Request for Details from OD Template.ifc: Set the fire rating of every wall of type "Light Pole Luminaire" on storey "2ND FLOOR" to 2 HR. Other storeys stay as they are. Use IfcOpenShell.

First a look at what the model holds.

```python
import ifcopenshell
import ifcopenshell.util.element

model = ifcopenshell.open("Details from OD Template.ifc")
print(model.schema)
storey = next(s for s in model.by_type("IfcBuildingStorey") if s.Name == "2ND FLOOR")
walls = [e for e in ifcopenshell.util.element.get_decomposition(storey) if e.is_a("IfcWall")]
seen = {}
for e in walls:
    element_type = ifcopenshell.util.element.get_type(e)
    key = (element_type.Name if element_type != e and element_type else None, ifcopenshell.util.element.get_pset(e, "Pset_WallCommon", "FireRating"))
    seen[key] = seen.get(key, 0) + 1
for (name, value), count in sorted(seen.items(), key=str):
    print(count, "x", name, "|", value)
```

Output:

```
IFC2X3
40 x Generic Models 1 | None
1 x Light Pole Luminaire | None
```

```python
import ifcopenshell
import ifcopenshell.api.pset
import ifcopenshell.util.element

model = ifcopenshell.open("Details from OD Template.ifc")

storey = next(s for s in model.by_type("IfcBuildingStorey") if s.Name == "2ND FLOOR")
walls = [e for e in ifcopenshell.util.element.get_decomposition(storey) if e.is_a("IfcWall")]

count = 0
for e in walls:
    element_type = ifcopenshell.util.element.get_type(e)
    if element_type in (None, e) or element_type.Name != "Light Pole Luminaire":
        continue
    # add_pset returns the element's existing set when there is one.
    pset = ifcopenshell.api.pset.add_pset(model, product=e, name="Pset_WallCommon")
    ifcopenshell.api.pset.edit_pset(model, pset=pset, properties={"FireRating": "2 HR"})
    count += 1

print(count, "walls updated")

model.write("Details from OD Template_edited.ifc")
```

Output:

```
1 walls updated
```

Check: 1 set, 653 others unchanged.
